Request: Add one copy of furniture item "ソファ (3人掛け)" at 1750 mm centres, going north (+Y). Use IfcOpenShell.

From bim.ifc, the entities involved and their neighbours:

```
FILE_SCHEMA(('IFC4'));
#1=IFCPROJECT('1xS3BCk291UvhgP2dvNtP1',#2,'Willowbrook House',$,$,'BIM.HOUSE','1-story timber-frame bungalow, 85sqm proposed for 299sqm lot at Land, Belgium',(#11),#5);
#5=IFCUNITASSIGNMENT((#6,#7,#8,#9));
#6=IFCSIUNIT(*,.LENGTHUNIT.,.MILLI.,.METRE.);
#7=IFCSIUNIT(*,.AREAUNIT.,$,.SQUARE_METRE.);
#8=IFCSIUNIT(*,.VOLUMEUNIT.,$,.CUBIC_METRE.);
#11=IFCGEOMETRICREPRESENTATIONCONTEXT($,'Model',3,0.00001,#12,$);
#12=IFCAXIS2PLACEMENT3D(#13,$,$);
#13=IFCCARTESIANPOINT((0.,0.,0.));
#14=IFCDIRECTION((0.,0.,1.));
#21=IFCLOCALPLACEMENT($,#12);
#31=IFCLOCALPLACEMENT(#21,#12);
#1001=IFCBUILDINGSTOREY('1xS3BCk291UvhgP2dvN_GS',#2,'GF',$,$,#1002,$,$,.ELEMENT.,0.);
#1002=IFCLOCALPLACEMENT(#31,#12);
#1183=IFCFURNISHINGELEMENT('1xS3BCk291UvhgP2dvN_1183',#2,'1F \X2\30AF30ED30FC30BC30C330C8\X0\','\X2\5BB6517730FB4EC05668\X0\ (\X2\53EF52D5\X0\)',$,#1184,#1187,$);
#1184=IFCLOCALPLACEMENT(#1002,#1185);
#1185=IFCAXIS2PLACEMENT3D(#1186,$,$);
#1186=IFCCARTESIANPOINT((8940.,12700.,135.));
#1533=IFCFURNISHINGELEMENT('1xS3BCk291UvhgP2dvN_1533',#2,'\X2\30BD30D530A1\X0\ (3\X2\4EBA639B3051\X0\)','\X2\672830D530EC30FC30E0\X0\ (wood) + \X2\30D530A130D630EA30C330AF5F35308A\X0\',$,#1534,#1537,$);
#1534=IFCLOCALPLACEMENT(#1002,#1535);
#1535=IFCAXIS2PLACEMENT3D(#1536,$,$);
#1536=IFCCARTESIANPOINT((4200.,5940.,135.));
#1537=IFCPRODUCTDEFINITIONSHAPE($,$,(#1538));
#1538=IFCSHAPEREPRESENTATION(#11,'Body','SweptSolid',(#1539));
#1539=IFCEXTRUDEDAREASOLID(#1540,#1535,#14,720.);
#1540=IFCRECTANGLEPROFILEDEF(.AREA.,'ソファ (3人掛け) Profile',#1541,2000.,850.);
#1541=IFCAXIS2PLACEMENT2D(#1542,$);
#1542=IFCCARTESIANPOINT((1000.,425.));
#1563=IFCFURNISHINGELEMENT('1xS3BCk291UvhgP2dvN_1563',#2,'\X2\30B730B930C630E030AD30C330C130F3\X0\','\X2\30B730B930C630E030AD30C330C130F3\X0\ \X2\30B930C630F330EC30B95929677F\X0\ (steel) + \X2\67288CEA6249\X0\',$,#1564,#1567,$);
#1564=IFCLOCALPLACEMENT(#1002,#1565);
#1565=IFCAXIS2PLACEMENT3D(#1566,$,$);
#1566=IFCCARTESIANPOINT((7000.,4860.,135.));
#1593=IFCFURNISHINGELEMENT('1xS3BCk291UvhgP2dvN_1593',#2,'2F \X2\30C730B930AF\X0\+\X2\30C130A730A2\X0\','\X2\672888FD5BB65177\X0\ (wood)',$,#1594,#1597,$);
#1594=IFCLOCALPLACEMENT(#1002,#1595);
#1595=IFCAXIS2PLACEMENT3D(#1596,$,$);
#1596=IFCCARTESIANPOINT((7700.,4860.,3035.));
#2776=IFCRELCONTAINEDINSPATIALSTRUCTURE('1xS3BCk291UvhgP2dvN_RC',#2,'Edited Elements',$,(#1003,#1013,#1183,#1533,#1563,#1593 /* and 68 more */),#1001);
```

```python
import numpy as np
import ifcopenshell
import ifcopenshell.api.geometry
import ifcopenshell.api.root
import ifcopenshell.util.element
import ifcopenshell.util.placement
import ifcopenshell.util.unit

model = ifcopenshell.open("bim.ifc")
unit_scale = ifcopenshell.util.unit.calculate_unit_scale(model)


def reuse_history(source, copy):
    """copy_class also copies each property set's owner history, people and application; keep the originals."""
    for rel in copy.IsDefinedBy:
        if rel.is_a("IfcRelDefinesByProperties") and (history := rel.RelatingPropertyDefinition.OwnerHistory):
            rel.RelatingPropertyDefinition.OwnerHistory = source.OwnerHistory
            ifcopenshell.util.element.remove_deep2(model, history)


source = model.by_id(1533)
base = ifcopenshell.util.placement.get_local_placement(source.ObjectPlacement)
step = np.array([0.0, 1.0, 0.0]) * 1.75 / unit_scale

for i in range(1, 2):
    copy = ifcopenshell.api.root.copy_class(model, product=source)
    copy.Representation = ifcopenshell.util.element.copy_deep(
        model, source.Representation, exclude=["IfcGeometricRepresentationContext", "IfcRepresentationMap"]
    )
    reuse_history(source, copy)
    matrix = base.copy()
    matrix[:3, 3] += i * step
    print("added at", matrix[:3, 3].round(3) + 0.0)
    ifcopenshell.api.geometry.edit_object_placement(model, product=copy, matrix=matrix, is_si=False)

model.write("bim_v2.ifc")
```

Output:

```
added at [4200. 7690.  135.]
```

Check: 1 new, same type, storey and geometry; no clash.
